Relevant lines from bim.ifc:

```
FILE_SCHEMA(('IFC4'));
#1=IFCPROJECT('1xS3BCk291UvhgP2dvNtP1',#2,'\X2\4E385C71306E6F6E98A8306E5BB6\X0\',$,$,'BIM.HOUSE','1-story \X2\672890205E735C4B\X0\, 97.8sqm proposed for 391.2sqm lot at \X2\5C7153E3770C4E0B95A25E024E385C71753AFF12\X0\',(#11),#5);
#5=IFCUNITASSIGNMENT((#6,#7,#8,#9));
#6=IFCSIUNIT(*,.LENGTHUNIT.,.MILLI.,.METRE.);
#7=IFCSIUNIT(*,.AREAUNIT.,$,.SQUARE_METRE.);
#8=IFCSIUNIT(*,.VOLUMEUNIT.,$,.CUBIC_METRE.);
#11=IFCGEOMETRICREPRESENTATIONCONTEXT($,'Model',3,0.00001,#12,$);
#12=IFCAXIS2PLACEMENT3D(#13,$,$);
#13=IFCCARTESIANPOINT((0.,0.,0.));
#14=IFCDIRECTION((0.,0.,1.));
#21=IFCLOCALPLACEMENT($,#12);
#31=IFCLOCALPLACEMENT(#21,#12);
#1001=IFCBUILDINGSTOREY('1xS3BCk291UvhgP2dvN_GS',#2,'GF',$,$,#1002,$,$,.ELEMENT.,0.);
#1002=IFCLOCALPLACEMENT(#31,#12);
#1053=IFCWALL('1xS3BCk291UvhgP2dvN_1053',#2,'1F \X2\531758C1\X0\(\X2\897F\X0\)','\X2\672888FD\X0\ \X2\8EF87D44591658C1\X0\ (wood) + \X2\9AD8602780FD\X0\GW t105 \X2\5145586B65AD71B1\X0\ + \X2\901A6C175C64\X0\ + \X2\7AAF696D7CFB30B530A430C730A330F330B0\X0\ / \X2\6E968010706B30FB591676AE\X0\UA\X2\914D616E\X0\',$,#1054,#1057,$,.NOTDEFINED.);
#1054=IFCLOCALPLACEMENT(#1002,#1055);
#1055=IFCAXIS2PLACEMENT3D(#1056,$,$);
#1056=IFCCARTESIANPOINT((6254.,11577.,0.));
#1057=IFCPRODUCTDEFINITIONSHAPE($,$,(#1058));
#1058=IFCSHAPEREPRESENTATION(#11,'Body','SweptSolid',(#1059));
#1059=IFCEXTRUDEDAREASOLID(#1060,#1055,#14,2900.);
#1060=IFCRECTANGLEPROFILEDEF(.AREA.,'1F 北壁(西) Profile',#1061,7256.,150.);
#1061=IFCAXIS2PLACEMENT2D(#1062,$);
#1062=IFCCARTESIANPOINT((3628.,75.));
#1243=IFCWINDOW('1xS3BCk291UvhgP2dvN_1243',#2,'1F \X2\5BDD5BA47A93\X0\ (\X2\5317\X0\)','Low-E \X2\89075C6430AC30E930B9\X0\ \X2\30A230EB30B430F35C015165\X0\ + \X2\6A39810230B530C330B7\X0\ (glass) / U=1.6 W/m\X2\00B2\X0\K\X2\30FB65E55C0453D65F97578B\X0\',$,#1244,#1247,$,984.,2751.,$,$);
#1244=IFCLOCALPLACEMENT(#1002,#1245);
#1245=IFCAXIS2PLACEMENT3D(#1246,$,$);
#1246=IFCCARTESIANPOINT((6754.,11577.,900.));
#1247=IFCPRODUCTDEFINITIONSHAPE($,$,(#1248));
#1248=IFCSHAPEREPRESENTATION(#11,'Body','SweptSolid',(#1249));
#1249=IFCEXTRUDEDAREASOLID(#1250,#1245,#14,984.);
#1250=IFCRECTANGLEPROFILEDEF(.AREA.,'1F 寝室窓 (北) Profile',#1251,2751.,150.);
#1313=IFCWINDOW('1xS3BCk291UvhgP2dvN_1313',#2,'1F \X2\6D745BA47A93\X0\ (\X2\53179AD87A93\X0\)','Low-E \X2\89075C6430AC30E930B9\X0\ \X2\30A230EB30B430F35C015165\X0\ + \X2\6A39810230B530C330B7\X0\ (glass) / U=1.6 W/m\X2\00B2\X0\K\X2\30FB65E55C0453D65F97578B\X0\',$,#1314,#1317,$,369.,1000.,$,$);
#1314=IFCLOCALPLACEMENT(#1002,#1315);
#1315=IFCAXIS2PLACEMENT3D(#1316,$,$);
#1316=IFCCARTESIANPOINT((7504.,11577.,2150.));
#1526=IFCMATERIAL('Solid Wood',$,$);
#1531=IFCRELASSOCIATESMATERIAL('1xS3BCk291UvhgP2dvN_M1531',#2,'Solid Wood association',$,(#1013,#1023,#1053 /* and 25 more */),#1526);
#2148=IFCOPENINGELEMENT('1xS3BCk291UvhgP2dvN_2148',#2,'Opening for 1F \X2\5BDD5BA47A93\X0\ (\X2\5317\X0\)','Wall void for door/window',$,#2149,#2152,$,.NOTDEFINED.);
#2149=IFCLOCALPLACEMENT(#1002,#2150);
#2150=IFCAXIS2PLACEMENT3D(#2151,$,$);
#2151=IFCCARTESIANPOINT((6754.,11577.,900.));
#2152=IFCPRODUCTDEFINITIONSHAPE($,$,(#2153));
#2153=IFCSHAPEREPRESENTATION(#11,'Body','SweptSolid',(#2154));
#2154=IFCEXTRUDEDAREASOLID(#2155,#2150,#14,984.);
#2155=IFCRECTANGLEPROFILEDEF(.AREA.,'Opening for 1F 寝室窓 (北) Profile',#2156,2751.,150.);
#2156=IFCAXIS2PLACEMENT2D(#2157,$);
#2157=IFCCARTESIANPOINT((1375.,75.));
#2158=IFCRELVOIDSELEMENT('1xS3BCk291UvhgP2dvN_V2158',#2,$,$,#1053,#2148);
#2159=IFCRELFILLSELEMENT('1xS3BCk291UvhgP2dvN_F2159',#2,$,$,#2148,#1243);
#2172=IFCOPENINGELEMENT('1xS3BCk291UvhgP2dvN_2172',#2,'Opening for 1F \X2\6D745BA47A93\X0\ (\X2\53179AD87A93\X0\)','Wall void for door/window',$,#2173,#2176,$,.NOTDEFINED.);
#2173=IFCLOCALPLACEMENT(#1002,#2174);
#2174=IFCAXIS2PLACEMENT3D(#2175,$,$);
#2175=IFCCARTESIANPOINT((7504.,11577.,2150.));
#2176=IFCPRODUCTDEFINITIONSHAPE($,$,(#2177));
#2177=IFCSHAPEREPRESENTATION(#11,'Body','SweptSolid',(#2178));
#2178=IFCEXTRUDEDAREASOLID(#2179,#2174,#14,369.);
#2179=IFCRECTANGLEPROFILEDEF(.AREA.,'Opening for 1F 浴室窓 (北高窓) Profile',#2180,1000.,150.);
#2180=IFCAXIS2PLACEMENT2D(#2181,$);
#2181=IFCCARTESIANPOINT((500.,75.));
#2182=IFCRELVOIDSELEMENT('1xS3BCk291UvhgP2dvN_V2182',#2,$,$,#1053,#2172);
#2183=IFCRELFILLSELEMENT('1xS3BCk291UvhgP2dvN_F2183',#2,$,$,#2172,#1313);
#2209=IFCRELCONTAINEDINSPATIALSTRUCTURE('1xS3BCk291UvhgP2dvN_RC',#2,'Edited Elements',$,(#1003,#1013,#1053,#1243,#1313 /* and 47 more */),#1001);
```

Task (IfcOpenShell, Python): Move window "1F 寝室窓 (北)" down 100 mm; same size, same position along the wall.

```python
import numpy as np
import ifcopenshell
import ifcopenshell.api.geometry
import ifcopenshell.util.placement
import ifcopenshell.util.unit

model = ifcopenshell.open("bim.ifc")
unit_scale = ifcopenshell.util.unit.calculate_unit_scale(model)

window = model.by_id(1243)
opening = window.FillsVoids[0].RelatingOpeningElement
dz = -100.0

shift = np.array([0.0, 0.0, dz])
# The window is not placed relative to its opening, so move both.
for product in (opening, window):
    matrix = ifcopenshell.util.placement.get_local_placement(product.ObjectPlacement)
    matrix[:3, 3] += shift
    ifcopenshell.api.geometry.edit_object_placement(model, product=product, matrix=matrix, is_si=False)

print(f"moved by {dz * unit_scale:+.3f} m")

model.write("bim_edited.ifc")
```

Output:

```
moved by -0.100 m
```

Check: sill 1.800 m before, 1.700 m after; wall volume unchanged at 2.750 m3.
